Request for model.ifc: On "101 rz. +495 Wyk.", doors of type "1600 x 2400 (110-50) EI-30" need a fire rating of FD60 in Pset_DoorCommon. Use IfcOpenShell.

First a look at what the model holds.

```python
import ifcopenshell
import ifcopenshell.util.element

model = ifcopenshell.open("model.ifc")
print(model.schema)
storey = next(s for s in model.by_type("IfcBuildingStorey") if s.Name == "101 rz. +495 Wyk.")
doors = [e for e in ifcopenshell.util.element.get_decomposition(storey) if e.is_a("IfcDoor")]
seen = {}
for e in doors:
    element_type = ifcopenshell.util.element.get_type(e)
    key = (element_type.Name if element_type != e and element_type else None, ifcopenshell.util.element.get_pset(e, "Pset_DoorCommon", "FireRating"))
    seen[key] = seen.get(key, 0) + 1
for (name, value), count in sorted(seen.items(), key=str):
    print(count, "x", name, "|", value)
```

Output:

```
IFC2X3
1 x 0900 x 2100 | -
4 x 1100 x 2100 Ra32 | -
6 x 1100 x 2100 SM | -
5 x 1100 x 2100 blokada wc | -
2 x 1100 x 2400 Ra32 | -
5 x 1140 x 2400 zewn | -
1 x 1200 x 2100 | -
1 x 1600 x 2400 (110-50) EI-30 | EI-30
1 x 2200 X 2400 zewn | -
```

```python
import ifcopenshell
import ifcopenshell.api.pset
import ifcopenshell.util.element

model = ifcopenshell.open("model.ifc")

storey = next(s for s in model.by_type("IfcBuildingStorey") if s.Name == "101 rz. +495 Wyk.")
doors = [e for e in ifcopenshell.util.element.get_decomposition(storey) if e.is_a("IfcDoor")]

count = 0
for e in doors:
    element_type = ifcopenshell.util.element.get_type(e)
    if element_type in (None, e) or element_type.Name != "1600 x 2400 (110-50) EI-30":
        continue
    # add_pset returns the element's existing set when there is one.
    pset = ifcopenshell.api.pset.add_pset(model, product=e, name="Pset_DoorCommon")
    ifcopenshell.api.pset.edit_pset(model, pset=pset, properties={"FireRating": "FD60"})
    count += 1

print(count, "doors updated")

model.write("model_edited.ifc")
```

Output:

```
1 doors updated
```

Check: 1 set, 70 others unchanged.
